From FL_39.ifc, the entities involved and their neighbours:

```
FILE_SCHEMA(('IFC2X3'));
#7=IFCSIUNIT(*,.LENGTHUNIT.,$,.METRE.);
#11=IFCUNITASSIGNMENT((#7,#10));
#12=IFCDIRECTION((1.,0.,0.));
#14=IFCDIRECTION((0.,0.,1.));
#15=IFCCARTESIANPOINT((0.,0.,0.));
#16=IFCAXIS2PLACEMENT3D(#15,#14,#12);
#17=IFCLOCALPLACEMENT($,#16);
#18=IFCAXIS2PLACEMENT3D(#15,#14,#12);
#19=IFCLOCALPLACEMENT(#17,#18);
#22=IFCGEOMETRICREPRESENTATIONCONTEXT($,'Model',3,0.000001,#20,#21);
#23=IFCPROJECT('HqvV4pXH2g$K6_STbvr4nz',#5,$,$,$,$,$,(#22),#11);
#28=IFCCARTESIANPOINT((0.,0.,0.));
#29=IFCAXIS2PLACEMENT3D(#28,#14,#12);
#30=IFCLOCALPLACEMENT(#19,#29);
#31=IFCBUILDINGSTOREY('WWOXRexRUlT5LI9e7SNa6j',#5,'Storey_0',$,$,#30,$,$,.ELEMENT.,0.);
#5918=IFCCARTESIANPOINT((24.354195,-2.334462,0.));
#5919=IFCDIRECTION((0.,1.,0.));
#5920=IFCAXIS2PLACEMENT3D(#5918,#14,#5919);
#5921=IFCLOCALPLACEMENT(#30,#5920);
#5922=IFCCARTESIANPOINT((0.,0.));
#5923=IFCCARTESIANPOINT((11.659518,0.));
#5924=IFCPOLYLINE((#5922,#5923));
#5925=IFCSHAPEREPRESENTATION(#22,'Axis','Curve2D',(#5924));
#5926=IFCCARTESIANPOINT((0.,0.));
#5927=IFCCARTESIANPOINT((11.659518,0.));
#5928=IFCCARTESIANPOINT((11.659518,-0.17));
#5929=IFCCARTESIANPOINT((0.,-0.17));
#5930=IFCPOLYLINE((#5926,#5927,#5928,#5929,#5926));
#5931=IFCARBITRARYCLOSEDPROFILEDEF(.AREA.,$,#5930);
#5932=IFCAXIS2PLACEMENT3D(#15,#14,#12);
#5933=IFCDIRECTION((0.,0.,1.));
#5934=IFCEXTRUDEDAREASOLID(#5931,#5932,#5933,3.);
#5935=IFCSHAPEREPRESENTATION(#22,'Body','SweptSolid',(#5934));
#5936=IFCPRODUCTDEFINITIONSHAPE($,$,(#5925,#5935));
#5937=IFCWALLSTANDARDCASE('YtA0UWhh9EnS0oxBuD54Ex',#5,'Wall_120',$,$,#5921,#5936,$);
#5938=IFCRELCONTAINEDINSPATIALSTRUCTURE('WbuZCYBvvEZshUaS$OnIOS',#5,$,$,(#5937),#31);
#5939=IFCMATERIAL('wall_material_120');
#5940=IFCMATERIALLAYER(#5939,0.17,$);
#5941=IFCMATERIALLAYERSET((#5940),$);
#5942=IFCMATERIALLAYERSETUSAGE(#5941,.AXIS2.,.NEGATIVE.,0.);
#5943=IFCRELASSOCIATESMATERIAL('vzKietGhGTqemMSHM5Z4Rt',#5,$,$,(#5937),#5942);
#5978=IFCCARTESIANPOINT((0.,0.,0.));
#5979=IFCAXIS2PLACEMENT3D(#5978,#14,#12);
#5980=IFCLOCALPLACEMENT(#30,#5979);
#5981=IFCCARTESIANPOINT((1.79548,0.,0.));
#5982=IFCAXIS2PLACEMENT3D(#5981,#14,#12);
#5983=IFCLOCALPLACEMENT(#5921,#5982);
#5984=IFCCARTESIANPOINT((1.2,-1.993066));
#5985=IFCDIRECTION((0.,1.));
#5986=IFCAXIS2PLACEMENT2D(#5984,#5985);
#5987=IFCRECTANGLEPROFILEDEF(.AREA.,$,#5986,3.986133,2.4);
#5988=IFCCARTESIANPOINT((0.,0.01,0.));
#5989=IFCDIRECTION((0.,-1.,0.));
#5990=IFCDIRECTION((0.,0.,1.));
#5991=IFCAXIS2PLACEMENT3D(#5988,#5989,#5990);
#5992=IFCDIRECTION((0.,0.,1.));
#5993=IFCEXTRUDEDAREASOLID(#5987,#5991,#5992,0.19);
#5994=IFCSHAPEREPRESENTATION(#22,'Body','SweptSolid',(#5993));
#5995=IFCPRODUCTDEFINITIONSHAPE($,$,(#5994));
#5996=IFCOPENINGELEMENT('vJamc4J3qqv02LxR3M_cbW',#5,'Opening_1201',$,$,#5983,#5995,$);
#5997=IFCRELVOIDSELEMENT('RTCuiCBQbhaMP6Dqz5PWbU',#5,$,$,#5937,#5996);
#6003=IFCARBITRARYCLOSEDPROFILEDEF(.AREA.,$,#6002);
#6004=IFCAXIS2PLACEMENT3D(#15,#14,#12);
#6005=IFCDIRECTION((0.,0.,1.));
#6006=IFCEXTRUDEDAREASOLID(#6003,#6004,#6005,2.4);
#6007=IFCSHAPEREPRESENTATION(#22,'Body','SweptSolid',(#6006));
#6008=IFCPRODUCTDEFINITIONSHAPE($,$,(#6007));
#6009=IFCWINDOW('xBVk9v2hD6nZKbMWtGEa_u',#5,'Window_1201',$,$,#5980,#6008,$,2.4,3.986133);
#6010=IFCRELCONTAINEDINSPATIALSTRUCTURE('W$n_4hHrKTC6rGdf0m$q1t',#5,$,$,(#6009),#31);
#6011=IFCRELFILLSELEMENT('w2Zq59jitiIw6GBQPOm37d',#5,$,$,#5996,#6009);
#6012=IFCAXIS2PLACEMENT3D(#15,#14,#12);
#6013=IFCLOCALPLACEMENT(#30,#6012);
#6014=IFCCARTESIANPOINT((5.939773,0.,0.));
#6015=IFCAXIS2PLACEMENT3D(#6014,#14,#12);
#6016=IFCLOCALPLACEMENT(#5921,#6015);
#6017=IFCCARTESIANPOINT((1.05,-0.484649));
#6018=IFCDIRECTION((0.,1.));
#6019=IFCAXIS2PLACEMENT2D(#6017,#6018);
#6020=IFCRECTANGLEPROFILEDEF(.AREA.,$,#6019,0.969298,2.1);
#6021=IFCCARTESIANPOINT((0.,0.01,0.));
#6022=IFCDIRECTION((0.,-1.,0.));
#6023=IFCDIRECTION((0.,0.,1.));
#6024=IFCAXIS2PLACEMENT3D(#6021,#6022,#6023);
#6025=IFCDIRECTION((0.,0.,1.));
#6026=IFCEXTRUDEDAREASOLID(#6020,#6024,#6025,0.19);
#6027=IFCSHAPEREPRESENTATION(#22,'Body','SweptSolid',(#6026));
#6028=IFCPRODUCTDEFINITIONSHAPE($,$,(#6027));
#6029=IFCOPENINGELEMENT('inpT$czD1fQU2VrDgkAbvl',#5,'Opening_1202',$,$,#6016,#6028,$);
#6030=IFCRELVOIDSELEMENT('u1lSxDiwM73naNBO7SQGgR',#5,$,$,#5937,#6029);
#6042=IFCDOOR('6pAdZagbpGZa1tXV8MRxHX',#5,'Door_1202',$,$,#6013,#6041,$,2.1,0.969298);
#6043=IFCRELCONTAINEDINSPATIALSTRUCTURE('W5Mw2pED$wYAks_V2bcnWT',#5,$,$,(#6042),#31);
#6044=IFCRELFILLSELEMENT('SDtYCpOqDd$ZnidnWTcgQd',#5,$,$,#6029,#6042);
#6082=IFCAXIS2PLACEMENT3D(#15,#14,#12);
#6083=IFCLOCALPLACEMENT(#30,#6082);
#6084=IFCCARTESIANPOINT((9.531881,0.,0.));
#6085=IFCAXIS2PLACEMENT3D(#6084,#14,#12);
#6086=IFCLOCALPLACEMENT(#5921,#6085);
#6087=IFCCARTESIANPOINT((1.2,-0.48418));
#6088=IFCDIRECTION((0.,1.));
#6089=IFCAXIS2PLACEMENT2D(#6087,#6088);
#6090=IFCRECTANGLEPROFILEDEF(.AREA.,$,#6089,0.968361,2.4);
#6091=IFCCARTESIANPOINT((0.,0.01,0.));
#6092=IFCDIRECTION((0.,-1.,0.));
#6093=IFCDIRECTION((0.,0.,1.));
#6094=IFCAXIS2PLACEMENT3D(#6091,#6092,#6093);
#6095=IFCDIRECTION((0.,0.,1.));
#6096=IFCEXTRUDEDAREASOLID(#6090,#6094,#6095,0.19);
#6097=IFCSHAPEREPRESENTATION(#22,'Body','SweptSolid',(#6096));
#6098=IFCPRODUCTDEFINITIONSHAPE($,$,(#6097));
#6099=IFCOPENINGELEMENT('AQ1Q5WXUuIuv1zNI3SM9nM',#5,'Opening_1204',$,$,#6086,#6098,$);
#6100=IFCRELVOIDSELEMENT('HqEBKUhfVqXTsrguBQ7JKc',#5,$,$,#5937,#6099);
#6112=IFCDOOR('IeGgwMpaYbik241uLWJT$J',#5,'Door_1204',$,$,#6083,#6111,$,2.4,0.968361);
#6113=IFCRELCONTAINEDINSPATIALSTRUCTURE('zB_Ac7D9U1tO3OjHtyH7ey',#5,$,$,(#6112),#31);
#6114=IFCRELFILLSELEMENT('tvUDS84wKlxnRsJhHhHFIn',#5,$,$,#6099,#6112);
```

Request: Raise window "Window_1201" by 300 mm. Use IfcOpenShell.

```python
import numpy as np
import ifcopenshell
import ifcopenshell.api.geometry
import ifcopenshell.util.placement
import ifcopenshell.util.unit

model = ifcopenshell.open("FL_39.ifc")
unit_scale = ifcopenshell.util.unit.calculate_unit_scale(model)

window = model.by_guid("xBVk9v2hD6nZKbMWtGEa_u")
opening = window.FillsVoids[0].RelatingOpeningElement
dz = 0.3

shift = np.array([0.0, 0.0, dz])
# The window is not placed relative to its opening, so move both.
for product in (opening, window):
    matrix = ifcopenshell.util.placement.get_local_placement(product.ObjectPlacement)
    matrix[:3, 3] += shift
    ifcopenshell.api.geometry.edit_object_placement(model, product=product, matrix=matrix, is_si=False)

print(f"moved by {dz * unit_scale:+.3f} m")

model.write("FL_39-out.ifc")
```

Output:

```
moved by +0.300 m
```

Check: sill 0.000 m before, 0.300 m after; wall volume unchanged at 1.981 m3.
